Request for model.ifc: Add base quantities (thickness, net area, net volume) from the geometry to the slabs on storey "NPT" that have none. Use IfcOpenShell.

First a look at what the model holds.

```python
import ifcopenshell
import ifcopenshell.util.element
import ifcopenshell.util.unit

model = ifcopenshell.open("model.ifc")
print(model.schema)
for unit_type in ("LENGTHUNIT", "AREAUNIT", "VOLUMEUNIT"):
    print(unit_type, ifcopenshell.util.unit.calculate_unit_scale(model, unit_type))
storey = next(s for s in model.by_type("IfcBuildingStorey") if s.Name == "NPT")
slabs = [e for e in ifcopenshell.util.element.get_decomposition(storey) if e.is_a("IfcSlab")]
for e in sorted(slabs, key=lambda e: e.id()):
    print(e.id(), e.is_a(), e.Name, list(ifcopenshell.util.element.get_psets(e, qtos_only=True)), sep=" | ")
```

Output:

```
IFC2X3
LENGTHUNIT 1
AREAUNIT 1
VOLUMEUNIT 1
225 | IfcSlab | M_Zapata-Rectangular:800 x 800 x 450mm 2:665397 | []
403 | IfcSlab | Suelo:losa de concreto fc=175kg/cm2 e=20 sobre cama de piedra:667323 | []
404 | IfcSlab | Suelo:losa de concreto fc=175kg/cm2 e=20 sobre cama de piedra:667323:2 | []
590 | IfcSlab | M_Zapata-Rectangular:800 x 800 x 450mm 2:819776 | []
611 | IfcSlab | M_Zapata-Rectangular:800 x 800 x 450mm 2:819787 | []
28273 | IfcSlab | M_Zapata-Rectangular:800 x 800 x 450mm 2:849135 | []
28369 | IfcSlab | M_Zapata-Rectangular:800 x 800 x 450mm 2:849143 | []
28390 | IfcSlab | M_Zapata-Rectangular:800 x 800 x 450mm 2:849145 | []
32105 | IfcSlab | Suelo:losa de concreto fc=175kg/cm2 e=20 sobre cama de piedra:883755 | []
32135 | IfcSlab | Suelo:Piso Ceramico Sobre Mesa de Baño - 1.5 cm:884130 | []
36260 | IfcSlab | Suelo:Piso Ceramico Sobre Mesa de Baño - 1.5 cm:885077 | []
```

```python
import ifcopenshell
import ifcopenshell.api.pset
import ifcopenshell.geom
import ifcopenshell.util.element
import ifcopenshell.util.shape
import ifcopenshell.util.unit

model = ifcopenshell.open("model.ifc")
unit_scale = ifcopenshell.util.unit.calculate_unit_scale(model)
area_scale = ifcopenshell.util.unit.calculate_unit_scale(model, "AREAUNIT")
volume_scale = ifcopenshell.util.unit.calculate_unit_scale(model, "VOLUMEUNIT")
settings = ifcopenshell.geom.settings()

storey = next(s for s in model.by_type("IfcBuildingStorey") if s.Name == "NPT")
slabs = [e for e in ifcopenshell.util.element.get_decomposition(storey) if e.is_a("IfcSlab")]

for e in sorted(slabs, key=lambda e: e.id()):
    if ifcopenshell.util.element.get_psets(e, qtos_only=True, should_inherit=False):
        continue
    # Geometry comes back in metres, in the element's own axes.
    shape = ifcopenshell.geom.create_shape(settings, e)
    values = {
        "Width": ifcopenshell.util.shape.get_z(shape.geometry) / unit_scale,
        "NetArea": ifcopenshell.util.shape.get_footprint_area(shape.geometry) / area_scale,
        "NetVolume": ifcopenshell.util.shape.get_volume(shape.geometry) / volume_scale,
    }
    qto = ifcopenshell.api.pset.add_qto(model, product=e, name="BaseQuantities")
    ifcopenshell.api.pset.edit_qto(model, qto=qto, properties=values)
    print(e.id(), {k: round(v, 3) for k, v in values.items()})

model.write("model_rev.ifc")
```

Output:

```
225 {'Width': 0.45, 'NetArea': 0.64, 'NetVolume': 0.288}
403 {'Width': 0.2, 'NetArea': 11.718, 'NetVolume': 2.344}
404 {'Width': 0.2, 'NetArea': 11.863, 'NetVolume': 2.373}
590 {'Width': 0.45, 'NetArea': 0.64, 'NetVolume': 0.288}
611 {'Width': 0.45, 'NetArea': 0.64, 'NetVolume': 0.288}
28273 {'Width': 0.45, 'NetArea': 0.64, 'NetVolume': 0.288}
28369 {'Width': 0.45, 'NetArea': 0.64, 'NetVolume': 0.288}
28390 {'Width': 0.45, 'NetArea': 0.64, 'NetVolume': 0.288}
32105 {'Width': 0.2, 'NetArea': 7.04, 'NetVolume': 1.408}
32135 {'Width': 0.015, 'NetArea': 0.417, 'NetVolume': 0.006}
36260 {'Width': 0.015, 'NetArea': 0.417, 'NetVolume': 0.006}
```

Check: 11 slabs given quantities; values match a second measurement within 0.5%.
